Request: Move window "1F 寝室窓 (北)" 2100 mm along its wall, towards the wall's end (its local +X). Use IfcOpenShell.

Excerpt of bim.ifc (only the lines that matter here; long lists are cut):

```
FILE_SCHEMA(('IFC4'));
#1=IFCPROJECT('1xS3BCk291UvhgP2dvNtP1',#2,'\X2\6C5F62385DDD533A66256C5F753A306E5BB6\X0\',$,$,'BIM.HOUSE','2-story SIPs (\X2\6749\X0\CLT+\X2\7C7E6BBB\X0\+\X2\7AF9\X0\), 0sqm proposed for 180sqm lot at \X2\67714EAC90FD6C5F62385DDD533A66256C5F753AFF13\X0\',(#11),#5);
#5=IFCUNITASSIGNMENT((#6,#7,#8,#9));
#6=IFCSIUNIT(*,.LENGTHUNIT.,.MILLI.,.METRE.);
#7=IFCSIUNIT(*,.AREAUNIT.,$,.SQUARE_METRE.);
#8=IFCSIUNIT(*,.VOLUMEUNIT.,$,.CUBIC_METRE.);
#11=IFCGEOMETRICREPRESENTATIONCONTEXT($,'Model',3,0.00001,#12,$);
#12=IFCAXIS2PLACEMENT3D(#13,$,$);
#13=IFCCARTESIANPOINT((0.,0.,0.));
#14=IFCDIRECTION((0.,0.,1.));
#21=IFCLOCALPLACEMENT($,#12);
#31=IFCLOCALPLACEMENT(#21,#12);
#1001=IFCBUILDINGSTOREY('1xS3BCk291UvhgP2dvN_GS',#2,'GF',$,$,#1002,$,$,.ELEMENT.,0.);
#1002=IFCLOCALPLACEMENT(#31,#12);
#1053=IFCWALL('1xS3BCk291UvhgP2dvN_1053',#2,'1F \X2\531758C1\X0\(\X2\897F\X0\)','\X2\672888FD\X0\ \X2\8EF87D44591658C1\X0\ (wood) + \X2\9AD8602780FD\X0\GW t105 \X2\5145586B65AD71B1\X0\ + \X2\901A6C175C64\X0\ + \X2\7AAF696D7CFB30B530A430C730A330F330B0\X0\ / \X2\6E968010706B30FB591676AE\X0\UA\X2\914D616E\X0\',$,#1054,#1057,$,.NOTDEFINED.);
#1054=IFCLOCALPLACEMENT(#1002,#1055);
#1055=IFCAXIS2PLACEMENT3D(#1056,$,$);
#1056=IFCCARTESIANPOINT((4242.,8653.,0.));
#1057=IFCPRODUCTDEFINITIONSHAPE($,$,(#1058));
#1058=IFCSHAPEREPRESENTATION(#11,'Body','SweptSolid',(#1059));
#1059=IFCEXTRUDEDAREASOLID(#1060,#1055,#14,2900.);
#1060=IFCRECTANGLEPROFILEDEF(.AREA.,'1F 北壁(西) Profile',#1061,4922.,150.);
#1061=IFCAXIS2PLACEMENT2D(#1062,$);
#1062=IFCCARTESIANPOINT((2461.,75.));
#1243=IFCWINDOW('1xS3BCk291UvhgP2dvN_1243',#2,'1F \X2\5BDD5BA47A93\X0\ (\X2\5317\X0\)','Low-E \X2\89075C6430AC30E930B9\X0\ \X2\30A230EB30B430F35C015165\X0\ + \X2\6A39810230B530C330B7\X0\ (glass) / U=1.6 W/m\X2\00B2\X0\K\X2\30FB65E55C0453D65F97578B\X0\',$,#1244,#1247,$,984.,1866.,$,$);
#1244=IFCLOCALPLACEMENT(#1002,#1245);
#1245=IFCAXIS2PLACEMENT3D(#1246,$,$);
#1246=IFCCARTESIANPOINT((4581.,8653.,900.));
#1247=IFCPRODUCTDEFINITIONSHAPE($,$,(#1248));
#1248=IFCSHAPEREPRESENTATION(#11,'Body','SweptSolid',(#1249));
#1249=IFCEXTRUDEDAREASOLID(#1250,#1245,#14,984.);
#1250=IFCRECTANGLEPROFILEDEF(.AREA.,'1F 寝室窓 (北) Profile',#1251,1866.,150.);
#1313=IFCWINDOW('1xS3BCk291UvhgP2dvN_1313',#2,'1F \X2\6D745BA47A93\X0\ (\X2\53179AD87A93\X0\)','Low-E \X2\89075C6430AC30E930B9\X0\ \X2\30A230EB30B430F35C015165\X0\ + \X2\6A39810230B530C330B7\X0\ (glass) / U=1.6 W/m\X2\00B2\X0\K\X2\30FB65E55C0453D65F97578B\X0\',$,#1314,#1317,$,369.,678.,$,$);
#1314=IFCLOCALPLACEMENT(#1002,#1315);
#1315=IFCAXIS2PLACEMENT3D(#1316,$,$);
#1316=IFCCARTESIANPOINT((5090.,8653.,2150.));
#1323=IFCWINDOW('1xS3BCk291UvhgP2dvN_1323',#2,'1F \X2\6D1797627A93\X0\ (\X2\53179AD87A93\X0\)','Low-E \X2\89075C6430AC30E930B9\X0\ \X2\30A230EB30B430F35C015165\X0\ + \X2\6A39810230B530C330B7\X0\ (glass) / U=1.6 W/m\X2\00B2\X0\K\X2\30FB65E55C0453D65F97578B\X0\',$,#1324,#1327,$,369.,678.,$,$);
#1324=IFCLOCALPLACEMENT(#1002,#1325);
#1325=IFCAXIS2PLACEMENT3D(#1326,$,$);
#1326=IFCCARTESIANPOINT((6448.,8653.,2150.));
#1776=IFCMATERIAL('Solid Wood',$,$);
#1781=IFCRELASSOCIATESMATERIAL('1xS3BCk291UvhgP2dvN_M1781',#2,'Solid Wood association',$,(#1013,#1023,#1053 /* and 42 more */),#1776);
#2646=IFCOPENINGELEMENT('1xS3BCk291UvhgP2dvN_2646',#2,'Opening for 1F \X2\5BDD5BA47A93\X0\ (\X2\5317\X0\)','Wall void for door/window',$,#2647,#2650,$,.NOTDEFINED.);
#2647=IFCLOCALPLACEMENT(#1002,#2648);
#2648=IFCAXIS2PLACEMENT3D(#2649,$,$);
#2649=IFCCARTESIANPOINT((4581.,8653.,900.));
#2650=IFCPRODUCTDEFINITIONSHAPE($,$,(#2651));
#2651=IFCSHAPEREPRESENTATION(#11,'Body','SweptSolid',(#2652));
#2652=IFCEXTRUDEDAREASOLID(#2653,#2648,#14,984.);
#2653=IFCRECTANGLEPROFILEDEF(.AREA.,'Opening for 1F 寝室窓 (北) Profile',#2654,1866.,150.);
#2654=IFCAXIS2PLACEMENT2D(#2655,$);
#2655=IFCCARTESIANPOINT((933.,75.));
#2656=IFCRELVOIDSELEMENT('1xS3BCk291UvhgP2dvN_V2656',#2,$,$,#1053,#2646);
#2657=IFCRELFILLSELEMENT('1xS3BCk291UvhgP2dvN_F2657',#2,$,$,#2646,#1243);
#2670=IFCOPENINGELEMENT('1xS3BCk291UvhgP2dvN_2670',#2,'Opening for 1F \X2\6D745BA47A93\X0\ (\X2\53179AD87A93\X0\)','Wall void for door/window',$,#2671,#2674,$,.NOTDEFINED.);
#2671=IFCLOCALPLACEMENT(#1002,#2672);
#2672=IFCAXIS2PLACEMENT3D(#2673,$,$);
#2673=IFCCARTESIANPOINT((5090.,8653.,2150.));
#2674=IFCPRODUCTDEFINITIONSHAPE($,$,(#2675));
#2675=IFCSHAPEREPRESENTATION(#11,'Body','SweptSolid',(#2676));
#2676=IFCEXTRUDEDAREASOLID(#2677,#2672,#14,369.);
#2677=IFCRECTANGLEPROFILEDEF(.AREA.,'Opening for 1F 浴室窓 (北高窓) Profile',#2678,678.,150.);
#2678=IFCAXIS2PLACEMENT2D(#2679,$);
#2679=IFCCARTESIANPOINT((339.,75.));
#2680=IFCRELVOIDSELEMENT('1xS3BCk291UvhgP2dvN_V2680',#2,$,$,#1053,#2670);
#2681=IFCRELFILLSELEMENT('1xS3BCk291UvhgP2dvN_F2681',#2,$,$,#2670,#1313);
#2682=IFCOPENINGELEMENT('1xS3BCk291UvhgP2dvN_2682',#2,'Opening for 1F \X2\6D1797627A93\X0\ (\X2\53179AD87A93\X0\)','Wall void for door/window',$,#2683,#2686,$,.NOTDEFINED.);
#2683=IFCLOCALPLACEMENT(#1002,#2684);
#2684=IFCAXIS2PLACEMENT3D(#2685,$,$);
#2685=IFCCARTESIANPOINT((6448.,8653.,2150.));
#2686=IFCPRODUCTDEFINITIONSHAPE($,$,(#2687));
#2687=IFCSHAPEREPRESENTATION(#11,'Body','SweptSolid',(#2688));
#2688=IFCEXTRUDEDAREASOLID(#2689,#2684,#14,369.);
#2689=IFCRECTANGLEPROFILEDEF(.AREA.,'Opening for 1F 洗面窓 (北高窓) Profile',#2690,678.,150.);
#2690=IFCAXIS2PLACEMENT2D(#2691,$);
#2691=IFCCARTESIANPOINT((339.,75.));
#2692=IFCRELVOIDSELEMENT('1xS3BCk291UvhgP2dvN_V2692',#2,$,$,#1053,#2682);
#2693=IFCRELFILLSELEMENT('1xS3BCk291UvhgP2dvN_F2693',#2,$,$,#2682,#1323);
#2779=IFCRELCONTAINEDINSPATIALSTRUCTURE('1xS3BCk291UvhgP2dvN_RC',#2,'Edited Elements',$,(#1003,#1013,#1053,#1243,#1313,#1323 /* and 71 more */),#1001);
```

```python
import ifcopenshell
import ifcopenshell.api.geometry
import ifcopenshell.util.placement

model = ifcopenshell.open("bim.ifc")

window = model.by_guid("1xS3BCk291UvhgP2dvN_1243")
opening = window.FillsVoids[0].RelatingOpeningElement
wall = opening.VoidsElements[0].RelatingBuildingElement

wall_matrix = ifcopenshell.util.placement.get_local_placement(wall.ObjectPlacement)
shift = wall_matrix[:3, 0] * 2100.0
before = ifcopenshell.util.placement.get_local_placement(window.ObjectPlacement)[:3, 3].copy()

# The window is not placed relative to its opening, so move both.
for product in (opening, window):
    matrix = ifcopenshell.util.placement.get_local_placement(product.ObjectPlacement)
    matrix[:3, 3] += shift
    ifcopenshell.api.geometry.edit_object_placement(model, product=product, matrix=matrix, is_si=False)

after = ifcopenshell.util.placement.get_local_placement(window.ObjectPlacement)[:3, 3]
print("window moved by", (after - before).round(3) + 0.0)

model.write("bim-out.ifc")
```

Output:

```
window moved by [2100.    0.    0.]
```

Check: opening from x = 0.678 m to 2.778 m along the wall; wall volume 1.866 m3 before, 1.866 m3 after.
